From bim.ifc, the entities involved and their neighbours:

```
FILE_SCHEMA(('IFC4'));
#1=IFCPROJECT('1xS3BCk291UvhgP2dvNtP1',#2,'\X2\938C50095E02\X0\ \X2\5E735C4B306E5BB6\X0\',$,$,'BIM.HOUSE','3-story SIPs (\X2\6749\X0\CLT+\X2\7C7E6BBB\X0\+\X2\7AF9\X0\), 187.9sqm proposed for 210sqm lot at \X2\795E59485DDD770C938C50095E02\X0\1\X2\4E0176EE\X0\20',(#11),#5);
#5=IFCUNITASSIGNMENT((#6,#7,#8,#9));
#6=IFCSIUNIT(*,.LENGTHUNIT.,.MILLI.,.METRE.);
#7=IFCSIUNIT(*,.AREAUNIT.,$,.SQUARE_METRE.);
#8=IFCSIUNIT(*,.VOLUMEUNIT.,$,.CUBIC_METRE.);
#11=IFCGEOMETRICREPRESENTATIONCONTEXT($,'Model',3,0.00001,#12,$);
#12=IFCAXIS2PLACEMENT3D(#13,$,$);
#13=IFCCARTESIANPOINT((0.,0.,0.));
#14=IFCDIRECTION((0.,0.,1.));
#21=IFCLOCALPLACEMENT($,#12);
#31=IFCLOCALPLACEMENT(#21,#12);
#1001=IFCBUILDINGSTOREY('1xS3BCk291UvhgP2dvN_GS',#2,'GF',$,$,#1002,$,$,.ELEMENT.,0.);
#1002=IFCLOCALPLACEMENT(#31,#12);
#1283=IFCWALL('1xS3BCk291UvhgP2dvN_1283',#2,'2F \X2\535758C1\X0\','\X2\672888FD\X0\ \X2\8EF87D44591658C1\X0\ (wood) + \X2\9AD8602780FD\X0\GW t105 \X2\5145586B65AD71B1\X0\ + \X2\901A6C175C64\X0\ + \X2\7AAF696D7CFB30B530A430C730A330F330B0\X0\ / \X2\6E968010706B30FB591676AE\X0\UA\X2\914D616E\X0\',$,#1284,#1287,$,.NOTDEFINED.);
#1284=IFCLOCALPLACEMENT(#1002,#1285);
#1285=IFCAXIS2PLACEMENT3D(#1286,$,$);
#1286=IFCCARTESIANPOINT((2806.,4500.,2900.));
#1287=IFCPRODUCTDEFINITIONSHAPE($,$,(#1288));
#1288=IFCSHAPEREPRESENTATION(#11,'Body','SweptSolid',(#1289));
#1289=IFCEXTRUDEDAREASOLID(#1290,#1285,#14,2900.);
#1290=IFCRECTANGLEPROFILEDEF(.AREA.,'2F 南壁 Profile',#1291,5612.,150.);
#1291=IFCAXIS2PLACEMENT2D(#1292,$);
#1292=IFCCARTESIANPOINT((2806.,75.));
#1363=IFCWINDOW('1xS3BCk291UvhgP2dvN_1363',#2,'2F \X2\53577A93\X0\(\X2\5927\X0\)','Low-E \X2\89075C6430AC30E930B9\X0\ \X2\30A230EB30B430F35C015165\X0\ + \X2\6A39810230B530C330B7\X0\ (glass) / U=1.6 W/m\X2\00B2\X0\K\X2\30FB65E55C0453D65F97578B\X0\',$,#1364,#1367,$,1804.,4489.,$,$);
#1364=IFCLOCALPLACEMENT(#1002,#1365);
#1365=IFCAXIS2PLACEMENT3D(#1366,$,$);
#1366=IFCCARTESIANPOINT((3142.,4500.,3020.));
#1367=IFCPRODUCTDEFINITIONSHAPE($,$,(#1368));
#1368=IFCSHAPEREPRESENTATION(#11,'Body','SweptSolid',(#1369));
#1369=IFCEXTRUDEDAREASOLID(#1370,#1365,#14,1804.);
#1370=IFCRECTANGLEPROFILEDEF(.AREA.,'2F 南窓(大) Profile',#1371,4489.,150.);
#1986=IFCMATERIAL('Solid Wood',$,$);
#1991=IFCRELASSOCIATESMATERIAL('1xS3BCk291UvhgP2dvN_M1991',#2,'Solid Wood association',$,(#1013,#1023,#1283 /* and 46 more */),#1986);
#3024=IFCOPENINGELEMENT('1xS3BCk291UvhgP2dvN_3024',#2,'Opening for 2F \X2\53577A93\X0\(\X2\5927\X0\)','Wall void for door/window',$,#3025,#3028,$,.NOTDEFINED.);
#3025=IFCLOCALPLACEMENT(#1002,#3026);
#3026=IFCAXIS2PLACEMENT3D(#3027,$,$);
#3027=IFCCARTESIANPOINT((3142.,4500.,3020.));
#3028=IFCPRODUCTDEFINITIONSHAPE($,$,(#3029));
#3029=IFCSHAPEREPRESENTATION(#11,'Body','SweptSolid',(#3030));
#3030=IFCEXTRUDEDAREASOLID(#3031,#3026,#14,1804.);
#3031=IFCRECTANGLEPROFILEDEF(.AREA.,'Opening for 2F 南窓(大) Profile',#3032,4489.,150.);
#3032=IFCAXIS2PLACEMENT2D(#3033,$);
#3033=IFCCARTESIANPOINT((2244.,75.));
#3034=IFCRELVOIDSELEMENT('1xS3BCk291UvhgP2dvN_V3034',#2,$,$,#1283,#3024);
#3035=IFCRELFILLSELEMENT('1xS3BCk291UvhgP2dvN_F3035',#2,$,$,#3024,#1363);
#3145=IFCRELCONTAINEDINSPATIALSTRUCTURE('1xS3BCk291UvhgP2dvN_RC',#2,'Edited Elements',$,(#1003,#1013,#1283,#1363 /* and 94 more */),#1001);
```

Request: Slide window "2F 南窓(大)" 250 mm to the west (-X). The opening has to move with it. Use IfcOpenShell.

```python
import ifcopenshell
import ifcopenshell.api.geometry
import ifcopenshell.util.placement
import ifcopenshell.util.unit

model = ifcopenshell.open("bim.ifc")
unit_scale = ifcopenshell.util.unit.calculate_unit_scale(model)

window = model.by_guid("1xS3BCk291UvhgP2dvN_1363")
opening = window.FillsVoids[0].RelatingOpeningElement
wall = opening.VoidsElements[0].RelatingBuildingElement

wall_matrix = ifcopenshell.util.placement.get_local_placement(wall.ObjectPlacement)
shift = wall_matrix[:3, 0] * -0.25 / unit_scale
before = ifcopenshell.util.placement.get_local_placement(window.ObjectPlacement)[:3, 3].copy()

# The window is not placed relative to its opening, so move both.
for product in (opening, window):
    matrix = ifcopenshell.util.placement.get_local_placement(product.ObjectPlacement)
    matrix[:3, 3] += shift
    ifcopenshell.api.geometry.edit_object_placement(model, product=product, matrix=matrix, is_si=False)

after = ifcopenshell.util.placement.get_local_placement(window.ObjectPlacement)[:3, 3]
print("window moved by", (after - before).round(3) + 0.0)

model.write("bim_updated.ifc")
```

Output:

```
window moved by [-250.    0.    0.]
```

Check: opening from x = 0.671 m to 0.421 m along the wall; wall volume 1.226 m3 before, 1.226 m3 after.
